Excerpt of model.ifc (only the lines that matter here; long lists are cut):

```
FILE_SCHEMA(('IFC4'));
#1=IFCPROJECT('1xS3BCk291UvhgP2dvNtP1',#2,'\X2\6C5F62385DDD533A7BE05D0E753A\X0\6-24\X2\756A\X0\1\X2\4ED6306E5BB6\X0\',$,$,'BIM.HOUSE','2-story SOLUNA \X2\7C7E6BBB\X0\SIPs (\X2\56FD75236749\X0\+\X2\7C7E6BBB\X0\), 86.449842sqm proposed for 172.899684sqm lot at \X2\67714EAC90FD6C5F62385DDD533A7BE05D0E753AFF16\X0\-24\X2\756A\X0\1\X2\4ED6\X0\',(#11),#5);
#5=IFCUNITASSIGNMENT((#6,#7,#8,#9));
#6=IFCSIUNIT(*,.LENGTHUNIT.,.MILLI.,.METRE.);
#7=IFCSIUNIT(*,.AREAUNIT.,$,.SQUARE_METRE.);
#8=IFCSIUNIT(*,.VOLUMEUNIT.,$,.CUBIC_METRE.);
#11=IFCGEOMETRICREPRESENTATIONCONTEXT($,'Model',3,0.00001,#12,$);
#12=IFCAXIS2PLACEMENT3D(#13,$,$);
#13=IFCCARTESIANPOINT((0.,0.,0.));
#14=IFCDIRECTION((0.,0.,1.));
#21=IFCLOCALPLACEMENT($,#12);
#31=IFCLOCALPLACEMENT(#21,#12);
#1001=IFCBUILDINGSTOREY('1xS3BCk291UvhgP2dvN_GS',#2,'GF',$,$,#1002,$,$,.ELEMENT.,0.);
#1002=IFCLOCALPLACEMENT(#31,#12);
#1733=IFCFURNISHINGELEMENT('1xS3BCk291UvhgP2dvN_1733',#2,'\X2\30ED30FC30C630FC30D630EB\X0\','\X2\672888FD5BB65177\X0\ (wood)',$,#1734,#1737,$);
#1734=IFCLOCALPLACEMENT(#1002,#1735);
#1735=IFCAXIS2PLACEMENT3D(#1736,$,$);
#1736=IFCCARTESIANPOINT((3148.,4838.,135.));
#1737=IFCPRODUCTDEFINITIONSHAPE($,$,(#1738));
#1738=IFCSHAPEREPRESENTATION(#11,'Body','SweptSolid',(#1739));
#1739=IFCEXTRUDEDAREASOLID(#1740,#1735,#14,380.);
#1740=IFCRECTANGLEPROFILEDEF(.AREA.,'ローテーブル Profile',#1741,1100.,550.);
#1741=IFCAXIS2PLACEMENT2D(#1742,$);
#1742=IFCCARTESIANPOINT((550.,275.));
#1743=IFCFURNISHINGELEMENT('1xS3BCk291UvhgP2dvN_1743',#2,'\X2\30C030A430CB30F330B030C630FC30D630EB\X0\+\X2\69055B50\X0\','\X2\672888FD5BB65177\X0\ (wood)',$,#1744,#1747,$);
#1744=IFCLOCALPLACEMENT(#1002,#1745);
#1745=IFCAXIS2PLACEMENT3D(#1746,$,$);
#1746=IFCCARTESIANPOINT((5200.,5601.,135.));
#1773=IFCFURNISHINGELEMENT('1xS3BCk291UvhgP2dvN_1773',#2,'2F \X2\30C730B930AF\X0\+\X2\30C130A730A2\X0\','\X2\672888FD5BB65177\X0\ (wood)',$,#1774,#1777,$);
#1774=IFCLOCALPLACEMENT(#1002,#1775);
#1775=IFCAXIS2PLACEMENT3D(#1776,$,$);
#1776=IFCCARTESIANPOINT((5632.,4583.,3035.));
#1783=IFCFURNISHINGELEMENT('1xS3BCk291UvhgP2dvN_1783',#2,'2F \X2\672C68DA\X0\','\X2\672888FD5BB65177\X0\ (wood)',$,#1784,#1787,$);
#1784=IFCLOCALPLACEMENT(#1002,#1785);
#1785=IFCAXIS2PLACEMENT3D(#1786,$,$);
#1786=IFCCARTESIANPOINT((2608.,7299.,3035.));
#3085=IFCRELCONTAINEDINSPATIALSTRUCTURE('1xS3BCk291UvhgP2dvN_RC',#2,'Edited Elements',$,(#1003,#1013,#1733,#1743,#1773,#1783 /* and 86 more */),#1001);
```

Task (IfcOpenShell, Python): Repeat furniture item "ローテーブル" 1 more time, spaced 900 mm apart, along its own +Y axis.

```python
import ifcopenshell
import ifcopenshell.api.geometry
import ifcopenshell.api.root
import ifcopenshell.util.element
import ifcopenshell.util.placement
import ifcopenshell.util.unit

model = ifcopenshell.open("model.ifc")
unit_scale = ifcopenshell.util.unit.calculate_unit_scale(model)


def reuse_history(source, copy):
    """copy_class also copies each property set's owner history, people and application; keep the originals."""
    for rel in copy.IsDefinedBy:
        if rel.is_a("IfcRelDefinesByProperties") and (history := rel.RelatingPropertyDefinition.OwnerHistory):
            rel.RelatingPropertyDefinition.OwnerHistory = source.OwnerHistory
            ifcopenshell.util.element.remove_deep2(model, history)


source = model.by_guid("1xS3BCk291UvhgP2dvN_1733")
base = ifcopenshell.util.placement.get_local_placement(source.ObjectPlacement)
step = base[:3, 1] * 0.9 / unit_scale

for i in range(1, 2):
    copy = ifcopenshell.api.root.copy_class(model, product=source)
    copy.Representation = ifcopenshell.util.element.copy_deep(
        model, source.Representation, exclude=["IfcGeometricRepresentationContext", "IfcRepresentationMap"]
    )
    reuse_history(source, copy)
    matrix = base.copy()
    matrix[:3, 3] += i * step
    print("added at", matrix[:3, 3].round(3) + 0.0)
    ifcopenshell.api.geometry.edit_object_placement(model, product=copy, matrix=matrix, is_si=False)

model.write("model_updated.ifc")
```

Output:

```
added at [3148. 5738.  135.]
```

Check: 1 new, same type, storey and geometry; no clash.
